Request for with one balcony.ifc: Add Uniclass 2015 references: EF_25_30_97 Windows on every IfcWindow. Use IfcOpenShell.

First a look at what the model holds.

```python
import ifcopenshell

model = ifcopenshell.open("with one balcony.ifc")
print(model.schema)
print("classifications:", [c.Name for c in model.by_type("IfcClassification")])
for ifc_class in ("IfcDoor", "IfcRoof", "IfcStair", "IfcWall", "IfcWindow"):
    print(ifc_class, len(model.by_type(ifc_class)))
```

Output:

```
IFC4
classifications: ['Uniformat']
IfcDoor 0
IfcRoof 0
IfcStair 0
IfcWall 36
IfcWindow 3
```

```python
import ifcopenshell
import ifcopenshell.api.classification

model = ifcopenshell.open("with one balcony.ifc")

system = ifcopenshell.api.classification.add_classification(model, classification="Uniclass 2015")

codes = {
    "IfcWindow": ("EF_25_30_97", "Windows"),
}
for ifc_class, (code, name) in codes.items():
    products = model.by_type(ifc_class)
    ifcopenshell.api.classification.add_reference(
        model, products=products, classification=system, identification=code, name=name
    )
    print(code, len(products))

model.write("with one balcony_updated.ifc")
```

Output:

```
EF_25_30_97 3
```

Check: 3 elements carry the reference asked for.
